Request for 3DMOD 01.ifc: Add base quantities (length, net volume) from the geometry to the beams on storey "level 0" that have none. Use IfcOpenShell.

First a look at what the model holds.

```python
import ifcopenshell
import ifcopenshell.util.element
import ifcopenshell.util.unit

model = ifcopenshell.open("3DMOD 01.ifc")
print(model.schema)
for unit_type in ("LENGTHUNIT", "AREAUNIT", "VOLUMEUNIT"):
    print(unit_type, ifcopenshell.util.unit.calculate_unit_scale(model, unit_type))
storey = next(s for s in model.by_type("IfcBuildingStorey") if s.Name == "level 0")
beams = [e for e in ifcopenshell.util.element.get_decomposition(storey) if e.is_a("IfcBeam")]
for e in sorted(beams, key=lambda e: e.id()):
    print(e.id(), e.is_a(), e.Name, list(ifcopenshell.util.element.get_psets(e, qtos_only=True)), sep=" | ")
```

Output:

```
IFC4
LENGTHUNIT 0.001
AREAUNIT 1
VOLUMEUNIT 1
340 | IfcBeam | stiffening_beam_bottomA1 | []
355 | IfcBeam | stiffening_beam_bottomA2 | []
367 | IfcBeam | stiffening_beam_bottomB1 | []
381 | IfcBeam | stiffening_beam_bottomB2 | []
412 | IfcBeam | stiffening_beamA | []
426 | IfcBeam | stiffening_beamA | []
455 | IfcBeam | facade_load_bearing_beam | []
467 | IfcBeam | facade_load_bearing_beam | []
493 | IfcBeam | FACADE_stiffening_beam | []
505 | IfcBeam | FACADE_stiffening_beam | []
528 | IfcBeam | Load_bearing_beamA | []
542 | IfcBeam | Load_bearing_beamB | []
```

```python
import ifcopenshell
import ifcopenshell.api.pset
import ifcopenshell.geom
import ifcopenshell.util.element
import ifcopenshell.util.shape
import ifcopenshell.util.unit

model = ifcopenshell.open("3DMOD 01.ifc")
unit_scale = ifcopenshell.util.unit.calculate_unit_scale(model)
volume_scale = ifcopenshell.util.unit.calculate_unit_scale(model, "VOLUMEUNIT")
settings = ifcopenshell.geom.settings()

storey = next(s for s in model.by_type("IfcBuildingStorey") if s.Name == "level 0")
beams = [e for e in ifcopenshell.util.element.get_decomposition(storey) if e.is_a("IfcBeam")]

for e in sorted(beams, key=lambda e: e.id()):
    if ifcopenshell.util.element.get_psets(e, qtos_only=True, should_inherit=False):
        continue
    # Geometry comes back in metres, in the element's own axes.
    shape = ifcopenshell.geom.create_shape(settings, e)
    values = {
        "Length": ifcopenshell.util.shape.get_max_xyz(shape.geometry) / unit_scale,
        "NetVolume": ifcopenshell.util.shape.get_volume(shape.geometry) / volume_scale,
    }
    qto = ifcopenshell.api.pset.add_qto(model, product=e, name="Qto_BeamBaseQuantities")
    ifcopenshell.api.pset.edit_qto(model, qto=qto, properties=values)
    print(e.id(), {k: round(v, 3) for k, v in values.items()})

model.write("3DMOD 01_edited.ifc")
```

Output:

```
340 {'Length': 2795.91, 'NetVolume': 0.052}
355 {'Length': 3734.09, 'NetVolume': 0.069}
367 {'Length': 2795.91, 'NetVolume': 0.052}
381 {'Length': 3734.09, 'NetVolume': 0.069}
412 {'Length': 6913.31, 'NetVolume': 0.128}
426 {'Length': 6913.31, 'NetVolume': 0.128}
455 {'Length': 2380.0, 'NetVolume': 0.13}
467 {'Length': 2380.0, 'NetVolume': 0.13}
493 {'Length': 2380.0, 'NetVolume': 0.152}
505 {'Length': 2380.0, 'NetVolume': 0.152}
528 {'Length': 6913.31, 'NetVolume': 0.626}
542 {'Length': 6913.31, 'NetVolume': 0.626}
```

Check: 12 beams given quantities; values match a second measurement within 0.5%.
